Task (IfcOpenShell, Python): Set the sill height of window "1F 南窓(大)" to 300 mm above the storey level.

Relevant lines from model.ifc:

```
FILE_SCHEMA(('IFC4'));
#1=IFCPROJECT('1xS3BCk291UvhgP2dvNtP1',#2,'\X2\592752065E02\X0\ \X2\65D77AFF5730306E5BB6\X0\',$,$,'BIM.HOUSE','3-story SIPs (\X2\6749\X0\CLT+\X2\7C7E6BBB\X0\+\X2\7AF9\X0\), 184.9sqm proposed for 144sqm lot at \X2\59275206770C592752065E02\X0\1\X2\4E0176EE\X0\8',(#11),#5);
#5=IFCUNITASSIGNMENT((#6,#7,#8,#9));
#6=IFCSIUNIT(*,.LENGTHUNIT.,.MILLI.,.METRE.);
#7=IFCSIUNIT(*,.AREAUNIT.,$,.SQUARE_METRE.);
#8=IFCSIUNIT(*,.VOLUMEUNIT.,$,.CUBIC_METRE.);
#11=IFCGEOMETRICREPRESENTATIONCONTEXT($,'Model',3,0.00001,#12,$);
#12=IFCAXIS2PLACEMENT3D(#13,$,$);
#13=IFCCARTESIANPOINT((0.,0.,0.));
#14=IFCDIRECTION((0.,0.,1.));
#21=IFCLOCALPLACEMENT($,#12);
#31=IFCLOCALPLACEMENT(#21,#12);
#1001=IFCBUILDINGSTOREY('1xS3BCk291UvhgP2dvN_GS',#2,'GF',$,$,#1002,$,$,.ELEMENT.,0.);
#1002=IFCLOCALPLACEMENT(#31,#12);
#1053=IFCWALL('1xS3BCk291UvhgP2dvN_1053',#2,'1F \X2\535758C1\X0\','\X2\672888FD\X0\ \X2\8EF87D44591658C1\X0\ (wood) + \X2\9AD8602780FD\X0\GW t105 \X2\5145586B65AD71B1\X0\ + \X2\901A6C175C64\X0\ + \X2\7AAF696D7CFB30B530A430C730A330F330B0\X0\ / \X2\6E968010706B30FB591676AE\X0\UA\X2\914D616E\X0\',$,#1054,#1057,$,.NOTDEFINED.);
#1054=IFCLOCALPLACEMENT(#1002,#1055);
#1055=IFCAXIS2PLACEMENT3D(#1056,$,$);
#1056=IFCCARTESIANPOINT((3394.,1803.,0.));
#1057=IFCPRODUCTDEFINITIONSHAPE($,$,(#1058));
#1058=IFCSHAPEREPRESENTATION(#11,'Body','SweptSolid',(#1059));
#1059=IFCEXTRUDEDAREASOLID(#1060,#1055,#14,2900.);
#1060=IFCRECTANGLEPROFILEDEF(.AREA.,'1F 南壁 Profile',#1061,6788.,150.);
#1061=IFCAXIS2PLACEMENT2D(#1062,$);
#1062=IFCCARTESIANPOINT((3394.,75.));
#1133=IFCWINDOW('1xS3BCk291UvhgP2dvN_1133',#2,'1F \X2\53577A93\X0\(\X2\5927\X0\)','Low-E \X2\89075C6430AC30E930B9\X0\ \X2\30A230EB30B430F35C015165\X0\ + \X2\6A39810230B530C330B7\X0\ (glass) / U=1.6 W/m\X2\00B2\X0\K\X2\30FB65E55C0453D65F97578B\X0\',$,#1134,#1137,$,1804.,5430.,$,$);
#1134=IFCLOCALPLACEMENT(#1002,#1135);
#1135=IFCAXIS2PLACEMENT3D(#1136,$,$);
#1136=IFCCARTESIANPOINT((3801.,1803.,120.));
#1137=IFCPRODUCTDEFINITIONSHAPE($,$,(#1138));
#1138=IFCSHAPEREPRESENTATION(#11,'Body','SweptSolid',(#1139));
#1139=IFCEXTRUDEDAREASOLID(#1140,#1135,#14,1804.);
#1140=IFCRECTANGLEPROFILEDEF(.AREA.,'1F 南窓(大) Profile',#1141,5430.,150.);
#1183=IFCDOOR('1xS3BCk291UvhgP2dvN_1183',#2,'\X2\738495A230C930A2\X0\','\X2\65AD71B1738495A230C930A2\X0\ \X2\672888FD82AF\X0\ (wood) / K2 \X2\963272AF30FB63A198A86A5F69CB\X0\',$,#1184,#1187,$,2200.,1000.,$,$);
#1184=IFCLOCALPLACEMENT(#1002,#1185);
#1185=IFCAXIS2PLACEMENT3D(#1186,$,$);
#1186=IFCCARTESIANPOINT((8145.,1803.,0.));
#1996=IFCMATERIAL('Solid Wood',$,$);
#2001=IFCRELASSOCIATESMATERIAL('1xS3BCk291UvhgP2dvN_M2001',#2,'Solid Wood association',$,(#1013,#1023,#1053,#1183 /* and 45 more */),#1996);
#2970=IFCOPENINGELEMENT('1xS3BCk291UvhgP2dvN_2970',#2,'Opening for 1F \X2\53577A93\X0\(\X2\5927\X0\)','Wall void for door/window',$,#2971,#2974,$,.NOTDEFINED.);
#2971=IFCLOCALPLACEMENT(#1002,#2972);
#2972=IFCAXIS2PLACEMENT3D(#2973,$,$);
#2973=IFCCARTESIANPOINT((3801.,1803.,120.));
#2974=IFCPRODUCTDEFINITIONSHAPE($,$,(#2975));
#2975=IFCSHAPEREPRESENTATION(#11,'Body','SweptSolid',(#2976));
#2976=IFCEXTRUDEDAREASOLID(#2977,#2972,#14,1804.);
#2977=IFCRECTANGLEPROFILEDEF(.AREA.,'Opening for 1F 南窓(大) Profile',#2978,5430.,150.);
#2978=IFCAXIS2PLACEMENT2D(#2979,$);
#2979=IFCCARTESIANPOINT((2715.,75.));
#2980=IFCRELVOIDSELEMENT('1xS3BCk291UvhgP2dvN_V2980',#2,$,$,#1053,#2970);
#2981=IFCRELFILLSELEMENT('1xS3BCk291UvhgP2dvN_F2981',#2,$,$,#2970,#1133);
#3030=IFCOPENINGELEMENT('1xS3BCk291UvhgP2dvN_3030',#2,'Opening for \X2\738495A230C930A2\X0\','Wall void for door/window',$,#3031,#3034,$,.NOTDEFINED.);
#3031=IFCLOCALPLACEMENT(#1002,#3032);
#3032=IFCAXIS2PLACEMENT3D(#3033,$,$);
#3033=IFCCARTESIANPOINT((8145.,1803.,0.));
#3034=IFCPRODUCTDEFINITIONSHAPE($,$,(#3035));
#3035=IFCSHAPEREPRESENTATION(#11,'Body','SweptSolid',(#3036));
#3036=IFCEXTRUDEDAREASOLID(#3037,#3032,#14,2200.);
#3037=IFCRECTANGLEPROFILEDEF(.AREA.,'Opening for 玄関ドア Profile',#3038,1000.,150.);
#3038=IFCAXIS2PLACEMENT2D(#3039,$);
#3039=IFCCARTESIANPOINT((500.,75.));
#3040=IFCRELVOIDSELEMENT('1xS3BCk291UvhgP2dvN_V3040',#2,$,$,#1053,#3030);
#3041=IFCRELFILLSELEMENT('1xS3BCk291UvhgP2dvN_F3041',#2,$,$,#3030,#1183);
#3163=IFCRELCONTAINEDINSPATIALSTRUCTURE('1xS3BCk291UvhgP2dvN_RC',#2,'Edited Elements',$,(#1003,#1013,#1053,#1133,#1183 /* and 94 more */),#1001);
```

```python
import numpy as np
import ifcopenshell
import ifcopenshell.api.geometry
import ifcopenshell.geom
import ifcopenshell.util.element
import ifcopenshell.util.placement
import ifcopenshell.util.shape
import ifcopenshell.util.unit

model = ifcopenshell.open("model.ifc")
unit_scale = ifcopenshell.util.unit.calculate_unit_scale(model)

window = model.by_id(1133)
opening = window.FillsVoids[0].RelatingOpeningElement
storey = ifcopenshell.util.element.get_container(window, ifc_class="IfcBuildingStorey")
level = ifcopenshell.util.placement.get_local_placement(storey.ObjectPlacement)[2, 3]

# The opening's origin need not be at the sill, so measure its lowest point.
shape = ifcopenshell.geom.create_shape(ifcopenshell.geom.settings(), opening)
bottom = ifcopenshell.util.shape.get_shape_bottom_elevation(shape, shape.geometry) / unit_scale
dz = level + 0.3 / unit_scale - bottom

shift = np.array([0.0, 0.0, dz])
# The window is not placed relative to its opening, so move both.
for product in (opening, window):
    matrix = ifcopenshell.util.placement.get_local_placement(product.ObjectPlacement)
    matrix[:3, 3] += shift
    ifcopenshell.api.geometry.edit_object_placement(model, product=product, matrix=matrix, is_si=False)

print(f"moved by {dz * unit_scale:+.3f} m")

model.write("model_rev.ifc")
```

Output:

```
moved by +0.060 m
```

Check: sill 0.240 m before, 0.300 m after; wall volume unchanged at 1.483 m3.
